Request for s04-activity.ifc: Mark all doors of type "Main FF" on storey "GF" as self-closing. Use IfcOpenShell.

First a look at what the model holds.

```python
import ifcopenshell
import ifcopenshell.util.element

model = ifcopenshell.open("s04-activity.ifc")
print(model.schema)
storey = next(s for s in model.by_type("IfcBuildingStorey") if s.Name == "GF")
doors = [e for e in ifcopenshell.util.element.get_decomposition(storey) if e.is_a("IfcDoor")]
seen = {}
for e in doors:
    element_type = ifcopenshell.util.element.get_type(e)
    key = (element_type.Name if element_type != e and element_type else None, ifcopenshell.util.element.get_pset(e, "Pset_DoorCommon", "SelfClosing"))
    seen[key] = seen.get(key, 0) + 1
for (name, value), count in sorted(seen.items(), key=str):
    print(count, "x", name, "|", value)
```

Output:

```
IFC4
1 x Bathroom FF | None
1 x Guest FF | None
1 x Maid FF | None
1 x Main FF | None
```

```python
import ifcopenshell
import ifcopenshell.api.pset
import ifcopenshell.util.element

model = ifcopenshell.open("s04-activity.ifc")

storey = next(s for s in model.by_type("IfcBuildingStorey") if s.Name == "GF")
doors = [e for e in ifcopenshell.util.element.get_decomposition(storey) if e.is_a("IfcDoor")]

count = 0
for e in doors:
    element_type = ifcopenshell.util.element.get_type(e)
    if element_type in (None, e) or element_type.Name != "Main FF":
        continue
    # add_pset returns the element's existing set when there is one.
    pset = ifcopenshell.api.pset.add_pset(model, product=e, name="Pset_DoorCommon")
    ifcopenshell.api.pset.edit_pset(model, pset=pset, properties={"SelfClosing": True})
    count += 1

print(count, "doors updated")

model.write("s04-activity_rev.ifc")
```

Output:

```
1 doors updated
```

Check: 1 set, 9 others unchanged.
